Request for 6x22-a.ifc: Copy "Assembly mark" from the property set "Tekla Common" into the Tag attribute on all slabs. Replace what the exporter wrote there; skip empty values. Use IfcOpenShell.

First a look at what the model holds.

```python
import ifcopenshell
import ifcopenshell.util.element

model = ifcopenshell.open("6x22-a.ifc")
print(model.schema)
slabs = model.by_type("IfcSlab")
print(len(slabs), "slabs")
for e in slabs[:8]:
    source = ifcopenshell.util.element.get_pset(e, "Tekla Common", "Assembly mark")
    target = e.Tag
    print(e.id(), repr(source), repr(target), sep=" | ")
```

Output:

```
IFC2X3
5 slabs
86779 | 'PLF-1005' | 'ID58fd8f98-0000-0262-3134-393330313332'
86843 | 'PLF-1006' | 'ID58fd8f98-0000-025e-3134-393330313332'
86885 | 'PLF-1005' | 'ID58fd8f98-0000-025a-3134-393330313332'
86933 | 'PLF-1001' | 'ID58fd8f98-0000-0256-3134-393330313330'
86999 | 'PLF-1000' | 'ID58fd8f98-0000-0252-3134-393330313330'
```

```python
import ifcopenshell
import ifcopenshell.util.element

model = ifcopenshell.open("6x22-a.ifc")

count = 0
for e in model.by_type("IfcSlab"):
    value = ifcopenshell.util.element.get_pset(e, "Tekla Common", "Assembly mark")
    current = e.Tag
    if not value or not value.strip() or current == value:
        continue
    e.Tag = value
    count += 1

print(count, "slabs updated")

model.write("6x22-a_v2.ifc")
```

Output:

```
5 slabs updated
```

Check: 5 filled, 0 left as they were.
